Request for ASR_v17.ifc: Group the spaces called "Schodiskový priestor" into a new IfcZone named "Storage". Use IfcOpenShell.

First a look at what the model holds.

```python
import ifcopenshell

model = ifcopenshell.open("ASR_v17.ifc")
print(model.schema)
seen = {}
for space in model.by_type("IfcSpace"):
    seen[space.LongName] = seen.get(space.LongName, 0) + 1
for name, count in sorted(seen.items(), key=str):
    print(count, "x", name)
print("zones:", [z.Name for z in model.by_type("IfcZone")][:20])
```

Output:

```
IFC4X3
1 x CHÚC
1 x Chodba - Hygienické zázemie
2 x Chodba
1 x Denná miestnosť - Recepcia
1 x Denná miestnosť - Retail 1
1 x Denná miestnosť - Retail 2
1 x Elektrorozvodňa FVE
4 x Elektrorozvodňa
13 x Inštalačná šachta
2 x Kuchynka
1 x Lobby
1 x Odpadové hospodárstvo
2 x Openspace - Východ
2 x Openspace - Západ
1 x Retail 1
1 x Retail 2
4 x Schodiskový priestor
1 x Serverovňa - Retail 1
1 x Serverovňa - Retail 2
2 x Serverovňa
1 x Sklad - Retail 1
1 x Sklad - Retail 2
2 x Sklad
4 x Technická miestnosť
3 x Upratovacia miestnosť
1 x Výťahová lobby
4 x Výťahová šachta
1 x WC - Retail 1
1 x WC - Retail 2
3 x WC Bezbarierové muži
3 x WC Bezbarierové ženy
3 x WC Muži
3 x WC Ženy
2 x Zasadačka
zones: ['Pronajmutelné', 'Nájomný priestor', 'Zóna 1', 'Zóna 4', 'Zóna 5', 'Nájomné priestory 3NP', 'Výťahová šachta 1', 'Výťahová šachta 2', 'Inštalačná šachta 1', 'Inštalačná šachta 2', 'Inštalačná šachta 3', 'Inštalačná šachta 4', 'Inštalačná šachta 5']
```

```python
import ifcopenshell
import ifcopenshell.api.group
import ifcopenshell.api.root

model = ifcopenshell.open("ASR_v17.ifc")

names = {"Schodiskový priestor"}
spaces = [s for s in model.by_type("IfcSpace") if s.LongName in names]

zone = ifcopenshell.api.root.create_entity(model, ifc_class="IfcZone", name="Storage")
ifcopenshell.api.group.assign_group(model, products=spaces, group=zone)
print(len(spaces), "spaces in", zone.Name)

model.write("ASR_v17_v2.ifc")
```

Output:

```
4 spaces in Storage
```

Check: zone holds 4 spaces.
